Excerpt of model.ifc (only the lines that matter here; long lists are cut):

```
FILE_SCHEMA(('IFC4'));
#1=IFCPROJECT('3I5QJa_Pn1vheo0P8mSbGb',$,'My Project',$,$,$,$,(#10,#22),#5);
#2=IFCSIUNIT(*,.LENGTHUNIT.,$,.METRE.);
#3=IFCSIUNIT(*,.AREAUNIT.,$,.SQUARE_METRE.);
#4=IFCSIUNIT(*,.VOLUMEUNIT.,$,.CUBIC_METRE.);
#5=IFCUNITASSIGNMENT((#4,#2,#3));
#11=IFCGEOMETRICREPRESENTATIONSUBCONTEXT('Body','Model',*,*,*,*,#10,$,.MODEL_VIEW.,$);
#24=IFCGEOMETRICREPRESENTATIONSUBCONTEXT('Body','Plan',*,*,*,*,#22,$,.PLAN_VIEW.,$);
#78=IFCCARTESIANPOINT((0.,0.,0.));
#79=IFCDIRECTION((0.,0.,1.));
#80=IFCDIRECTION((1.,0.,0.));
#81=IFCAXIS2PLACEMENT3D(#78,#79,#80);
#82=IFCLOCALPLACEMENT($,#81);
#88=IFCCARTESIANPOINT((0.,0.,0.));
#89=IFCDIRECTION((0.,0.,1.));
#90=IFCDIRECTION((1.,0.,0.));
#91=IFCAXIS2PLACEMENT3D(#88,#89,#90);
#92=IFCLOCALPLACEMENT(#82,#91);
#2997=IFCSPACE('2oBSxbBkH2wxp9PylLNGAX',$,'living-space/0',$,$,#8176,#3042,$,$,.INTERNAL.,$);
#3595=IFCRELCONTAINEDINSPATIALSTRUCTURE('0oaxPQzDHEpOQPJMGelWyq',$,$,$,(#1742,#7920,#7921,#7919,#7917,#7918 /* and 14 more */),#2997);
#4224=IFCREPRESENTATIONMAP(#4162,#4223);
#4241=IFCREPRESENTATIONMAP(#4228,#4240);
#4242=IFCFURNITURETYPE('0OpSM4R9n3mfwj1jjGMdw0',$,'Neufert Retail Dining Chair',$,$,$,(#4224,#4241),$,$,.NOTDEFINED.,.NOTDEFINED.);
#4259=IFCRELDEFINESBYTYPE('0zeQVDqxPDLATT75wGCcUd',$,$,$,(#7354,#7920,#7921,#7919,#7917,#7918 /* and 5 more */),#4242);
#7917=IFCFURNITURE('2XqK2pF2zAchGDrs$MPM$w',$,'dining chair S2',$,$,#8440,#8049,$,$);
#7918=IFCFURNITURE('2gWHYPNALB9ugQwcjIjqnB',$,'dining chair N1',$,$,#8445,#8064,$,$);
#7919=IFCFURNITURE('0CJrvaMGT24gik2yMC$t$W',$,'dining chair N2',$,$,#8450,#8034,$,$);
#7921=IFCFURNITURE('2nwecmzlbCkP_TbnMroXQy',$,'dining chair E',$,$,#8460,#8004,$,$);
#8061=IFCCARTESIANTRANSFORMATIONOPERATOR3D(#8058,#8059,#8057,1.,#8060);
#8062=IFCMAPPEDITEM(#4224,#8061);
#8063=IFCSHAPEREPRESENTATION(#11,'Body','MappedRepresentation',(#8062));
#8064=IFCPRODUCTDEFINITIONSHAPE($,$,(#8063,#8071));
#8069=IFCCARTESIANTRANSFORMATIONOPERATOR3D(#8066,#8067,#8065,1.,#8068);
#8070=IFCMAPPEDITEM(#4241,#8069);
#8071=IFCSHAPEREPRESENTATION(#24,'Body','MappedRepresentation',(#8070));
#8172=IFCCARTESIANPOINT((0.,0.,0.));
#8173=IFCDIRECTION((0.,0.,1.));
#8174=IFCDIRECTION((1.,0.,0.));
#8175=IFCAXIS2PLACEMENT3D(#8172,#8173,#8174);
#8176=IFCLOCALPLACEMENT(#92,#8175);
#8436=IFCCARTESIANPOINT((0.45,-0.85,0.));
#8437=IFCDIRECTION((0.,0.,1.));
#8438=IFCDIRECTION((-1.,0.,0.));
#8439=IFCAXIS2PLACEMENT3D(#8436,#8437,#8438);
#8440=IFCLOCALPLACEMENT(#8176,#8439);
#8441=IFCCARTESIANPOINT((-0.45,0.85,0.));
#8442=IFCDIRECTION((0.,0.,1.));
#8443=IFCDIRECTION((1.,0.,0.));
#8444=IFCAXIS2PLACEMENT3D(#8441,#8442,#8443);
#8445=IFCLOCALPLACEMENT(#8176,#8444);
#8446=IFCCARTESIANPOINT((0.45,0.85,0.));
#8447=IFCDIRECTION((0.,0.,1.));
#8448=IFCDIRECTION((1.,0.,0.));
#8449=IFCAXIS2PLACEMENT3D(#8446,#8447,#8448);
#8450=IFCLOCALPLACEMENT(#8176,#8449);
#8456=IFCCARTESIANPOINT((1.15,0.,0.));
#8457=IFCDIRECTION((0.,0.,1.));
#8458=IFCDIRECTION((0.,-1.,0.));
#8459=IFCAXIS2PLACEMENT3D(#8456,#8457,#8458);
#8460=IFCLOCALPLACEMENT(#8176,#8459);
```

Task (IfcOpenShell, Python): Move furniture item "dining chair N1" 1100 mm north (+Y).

```python
import ifcopenshell
import ifcopenshell.api.geometry
import ifcopenshell.util.placement
import ifcopenshell.util.unit

model = ifcopenshell.open("model.ifc")
unit_scale = ifcopenshell.util.unit.calculate_unit_scale(model)

item = model.by_guid("2gWHYPNALB9ugQwcjIjqnB")
matrix = ifcopenshell.util.placement.get_local_placement(item.ObjectPlacement)
matrix[1, 3] += 1.1 / unit_scale
ifcopenshell.api.geometry.edit_object_placement(model, product=item, matrix=matrix, is_si=False)

print(ifcopenshell.util.placement.get_local_placement(item.ObjectPlacement).round(3) + 0.0)

model.write("model_v2.ifc")
```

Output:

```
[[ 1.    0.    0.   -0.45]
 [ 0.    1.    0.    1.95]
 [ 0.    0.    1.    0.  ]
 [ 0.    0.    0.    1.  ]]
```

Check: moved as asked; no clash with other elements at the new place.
